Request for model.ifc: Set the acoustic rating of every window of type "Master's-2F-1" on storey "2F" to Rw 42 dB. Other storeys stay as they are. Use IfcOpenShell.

First a look at what the model holds.

```python
import ifcopenshell
import ifcopenshell.util.element

model = ifcopenshell.open("model.ifc")
print(model.schema)
storey = next(s for s in model.by_type("IfcBuildingStorey") if s.Name == "2F")
windows = [e for e in ifcopenshell.util.element.get_decomposition(storey) if e.is_a("IfcWindow")]
seen = {}
for e in windows:
    element_type = ifcopenshell.util.element.get_type(e)
    key = (element_type.Name if element_type != e and element_type else None, ifcopenshell.util.element.get_pset(e, "Pset_WindowCommon", "AcousticRating"))
    seen[key] = seen.get(key, 0) + 1
for (name, value), count in sorted(seen.items(), key=str):
    print(count, "x", name, "|", value)
```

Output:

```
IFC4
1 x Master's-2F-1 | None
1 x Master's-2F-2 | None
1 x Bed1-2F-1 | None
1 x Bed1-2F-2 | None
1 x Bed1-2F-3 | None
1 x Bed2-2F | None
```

```python
import ifcopenshell
import ifcopenshell.api.pset
import ifcopenshell.util.element

model = ifcopenshell.open("model.ifc")

storey = next(s for s in model.by_type("IfcBuildingStorey") if s.Name == "2F")
windows = [e for e in ifcopenshell.util.element.get_decomposition(storey) if e.is_a("IfcWindow")]

count = 0
for e in windows:
    element_type = ifcopenshell.util.element.get_type(e)
    if element_type in (None, e) or element_type.Name != "Master's-2F-1":
        continue
    # add_pset returns the element's existing set when there is one.
    pset = ifcopenshell.api.pset.add_pset(model, product=e, name="Pset_WindowCommon")
    ifcopenshell.api.pset.edit_pset(model, pset=pset, properties={"AcousticRating": "Rw 42 dB"})
    count += 1

print(count, "windows updated")

model.write("model-out.ifc")
```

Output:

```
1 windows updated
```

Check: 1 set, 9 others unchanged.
